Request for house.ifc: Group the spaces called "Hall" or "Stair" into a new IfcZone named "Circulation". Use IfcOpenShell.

First a look at what the model holds.

```python
import ifcopenshell

model = ifcopenshell.open("house.ifc")
print(model.schema)
seen = {}
for space in model.by_type("IfcSpace"):
    seen[space.LongName] = seen.get(space.LongName, 0) + 1
for name, count in sorted(seen.items(), key=str):
    print(count, "x", name)
print("zones:", [z.Name for z in model.by_type("IfcZone")][:20])
```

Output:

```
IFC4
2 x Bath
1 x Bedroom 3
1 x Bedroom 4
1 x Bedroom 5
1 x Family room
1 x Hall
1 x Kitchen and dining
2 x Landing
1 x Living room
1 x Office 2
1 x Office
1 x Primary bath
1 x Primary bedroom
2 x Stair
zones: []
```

```python
import ifcopenshell
import ifcopenshell.api.group
import ifcopenshell.api.root

model = ifcopenshell.open("house.ifc")

names = {"Hall", "Stair"}
spaces = [s for s in model.by_type("IfcSpace") if s.LongName in names]

zone = ifcopenshell.api.root.create_entity(model, ifc_class="IfcZone", name="Circulation")
ifcopenshell.api.group.assign_group(model, products=spaces, group=zone)
print(len(spaces), "spaces in", zone.Name)

model.write("house_updated.ifc")
```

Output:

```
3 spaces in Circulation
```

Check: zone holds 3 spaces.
